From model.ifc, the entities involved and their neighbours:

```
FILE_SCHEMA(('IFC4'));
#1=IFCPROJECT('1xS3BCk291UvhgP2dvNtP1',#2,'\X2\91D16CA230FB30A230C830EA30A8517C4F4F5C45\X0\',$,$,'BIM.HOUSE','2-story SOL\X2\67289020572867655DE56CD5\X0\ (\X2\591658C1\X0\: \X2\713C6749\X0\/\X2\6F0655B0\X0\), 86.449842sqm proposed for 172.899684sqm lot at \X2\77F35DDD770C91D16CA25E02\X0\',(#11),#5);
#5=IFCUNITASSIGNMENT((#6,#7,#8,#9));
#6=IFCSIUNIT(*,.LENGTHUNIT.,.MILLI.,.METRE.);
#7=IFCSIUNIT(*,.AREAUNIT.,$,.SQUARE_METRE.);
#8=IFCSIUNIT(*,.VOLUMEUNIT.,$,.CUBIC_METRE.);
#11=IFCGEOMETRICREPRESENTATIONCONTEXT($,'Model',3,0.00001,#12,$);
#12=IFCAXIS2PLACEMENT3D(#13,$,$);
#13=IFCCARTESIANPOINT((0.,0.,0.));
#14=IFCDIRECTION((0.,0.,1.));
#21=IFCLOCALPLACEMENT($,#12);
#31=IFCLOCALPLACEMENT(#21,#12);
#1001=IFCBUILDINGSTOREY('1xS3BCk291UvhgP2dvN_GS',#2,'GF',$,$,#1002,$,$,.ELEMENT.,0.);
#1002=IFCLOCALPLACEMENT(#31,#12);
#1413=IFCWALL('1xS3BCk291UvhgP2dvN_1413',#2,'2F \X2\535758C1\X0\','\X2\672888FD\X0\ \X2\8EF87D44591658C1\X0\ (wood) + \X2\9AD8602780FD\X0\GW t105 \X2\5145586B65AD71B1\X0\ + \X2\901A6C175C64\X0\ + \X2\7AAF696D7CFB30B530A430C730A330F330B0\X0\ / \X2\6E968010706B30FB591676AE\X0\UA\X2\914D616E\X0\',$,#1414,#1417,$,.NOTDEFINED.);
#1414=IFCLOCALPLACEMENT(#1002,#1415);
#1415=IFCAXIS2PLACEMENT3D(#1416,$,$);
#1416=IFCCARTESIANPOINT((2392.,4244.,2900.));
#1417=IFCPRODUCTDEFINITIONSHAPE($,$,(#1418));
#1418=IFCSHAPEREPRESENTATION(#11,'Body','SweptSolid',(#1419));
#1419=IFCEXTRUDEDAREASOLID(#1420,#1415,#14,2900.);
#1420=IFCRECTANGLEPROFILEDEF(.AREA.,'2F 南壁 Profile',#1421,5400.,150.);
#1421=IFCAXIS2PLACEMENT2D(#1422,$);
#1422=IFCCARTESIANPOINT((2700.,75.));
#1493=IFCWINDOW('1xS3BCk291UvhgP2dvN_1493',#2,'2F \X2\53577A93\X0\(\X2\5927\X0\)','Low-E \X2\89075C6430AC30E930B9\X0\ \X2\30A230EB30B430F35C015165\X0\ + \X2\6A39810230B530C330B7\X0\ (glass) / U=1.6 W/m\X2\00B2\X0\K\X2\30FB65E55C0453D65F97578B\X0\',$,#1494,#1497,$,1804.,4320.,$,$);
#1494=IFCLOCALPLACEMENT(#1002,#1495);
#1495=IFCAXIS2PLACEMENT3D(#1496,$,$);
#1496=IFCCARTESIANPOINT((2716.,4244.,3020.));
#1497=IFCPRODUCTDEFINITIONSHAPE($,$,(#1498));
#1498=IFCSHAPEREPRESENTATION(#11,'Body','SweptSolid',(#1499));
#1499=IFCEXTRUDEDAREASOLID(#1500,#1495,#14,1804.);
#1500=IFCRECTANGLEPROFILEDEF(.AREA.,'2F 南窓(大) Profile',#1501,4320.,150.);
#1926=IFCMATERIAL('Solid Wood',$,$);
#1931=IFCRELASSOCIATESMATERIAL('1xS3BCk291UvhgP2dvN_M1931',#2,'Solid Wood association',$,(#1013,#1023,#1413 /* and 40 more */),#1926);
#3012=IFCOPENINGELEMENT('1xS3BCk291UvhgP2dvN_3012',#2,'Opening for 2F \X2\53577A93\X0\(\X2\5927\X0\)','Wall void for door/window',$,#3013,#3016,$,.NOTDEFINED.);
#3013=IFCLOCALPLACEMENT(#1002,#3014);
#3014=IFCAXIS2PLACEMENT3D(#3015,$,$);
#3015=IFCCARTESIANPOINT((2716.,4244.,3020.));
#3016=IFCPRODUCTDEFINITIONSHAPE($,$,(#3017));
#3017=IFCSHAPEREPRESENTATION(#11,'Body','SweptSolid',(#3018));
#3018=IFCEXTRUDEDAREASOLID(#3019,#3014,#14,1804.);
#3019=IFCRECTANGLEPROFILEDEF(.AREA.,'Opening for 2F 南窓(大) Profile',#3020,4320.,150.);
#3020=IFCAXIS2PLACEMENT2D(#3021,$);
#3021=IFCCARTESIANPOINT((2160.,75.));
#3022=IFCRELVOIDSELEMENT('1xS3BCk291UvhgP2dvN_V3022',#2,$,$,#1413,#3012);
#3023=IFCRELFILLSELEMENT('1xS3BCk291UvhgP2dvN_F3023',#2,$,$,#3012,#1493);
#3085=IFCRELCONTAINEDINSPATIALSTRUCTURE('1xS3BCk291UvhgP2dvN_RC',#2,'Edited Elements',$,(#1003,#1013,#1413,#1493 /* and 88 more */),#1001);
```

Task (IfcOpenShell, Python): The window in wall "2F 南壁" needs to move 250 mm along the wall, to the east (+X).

```python
import ifcopenshell
import ifcopenshell.api.geometry
import ifcopenshell.util.placement

model = ifcopenshell.open("model.ifc")

window = model.by_guid("1xS3BCk291UvhgP2dvN_1493")
opening = window.FillsVoids[0].RelatingOpeningElement
wall = opening.VoidsElements[0].RelatingBuildingElement

wall_matrix = ifcopenshell.util.placement.get_local_placement(wall.ObjectPlacement)
shift = wall_matrix[:3, 0] * 250.0
before = ifcopenshell.util.placement.get_local_placement(window.ObjectPlacement)[:3, 3].copy()

# The window is not placed relative to its opening, so move both.
for product in (opening, window):
    matrix = ifcopenshell.util.placement.get_local_placement(product.ObjectPlacement)
    matrix[:3, 3] += shift
    ifcopenshell.api.geometry.edit_object_placement(model, product=product, matrix=matrix, is_si=False)

after = ifcopenshell.util.placement.get_local_placement(window.ObjectPlacement)[:3, 3]
print("window moved by", (after - before).round(3) + 0.0)

model.write("model-out.ifc")
```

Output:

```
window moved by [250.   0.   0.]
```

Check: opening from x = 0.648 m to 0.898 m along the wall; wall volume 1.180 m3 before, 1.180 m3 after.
